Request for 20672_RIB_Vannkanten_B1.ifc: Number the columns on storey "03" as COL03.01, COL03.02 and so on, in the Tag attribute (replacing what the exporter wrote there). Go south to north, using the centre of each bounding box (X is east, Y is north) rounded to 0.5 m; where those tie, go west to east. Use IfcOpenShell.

First a look at what the model holds.

```python
import ifcopenshell
import ifcopenshell.util.element
import ifcopenshell.util.placement

model = ifcopenshell.open("20672_RIB_Vannkanten_B1.ifc")
print(model.schema)
storey = next(s for s in model.by_type("IfcBuildingStorey") if s.Name == "03")
columns = [e for e in ifcopenshell.util.element.get_decomposition(storey) if e.is_a("IfcColumn")]
for e in sorted(columns, key=lambda e: e.id()):
    origin = ifcopenshell.util.placement.get_local_placement(e.ObjectPlacement)[:3, 3]
    print(e.id(), e.Tag, e.Name, origin.round(2) + 0.0, sep=" | ")
```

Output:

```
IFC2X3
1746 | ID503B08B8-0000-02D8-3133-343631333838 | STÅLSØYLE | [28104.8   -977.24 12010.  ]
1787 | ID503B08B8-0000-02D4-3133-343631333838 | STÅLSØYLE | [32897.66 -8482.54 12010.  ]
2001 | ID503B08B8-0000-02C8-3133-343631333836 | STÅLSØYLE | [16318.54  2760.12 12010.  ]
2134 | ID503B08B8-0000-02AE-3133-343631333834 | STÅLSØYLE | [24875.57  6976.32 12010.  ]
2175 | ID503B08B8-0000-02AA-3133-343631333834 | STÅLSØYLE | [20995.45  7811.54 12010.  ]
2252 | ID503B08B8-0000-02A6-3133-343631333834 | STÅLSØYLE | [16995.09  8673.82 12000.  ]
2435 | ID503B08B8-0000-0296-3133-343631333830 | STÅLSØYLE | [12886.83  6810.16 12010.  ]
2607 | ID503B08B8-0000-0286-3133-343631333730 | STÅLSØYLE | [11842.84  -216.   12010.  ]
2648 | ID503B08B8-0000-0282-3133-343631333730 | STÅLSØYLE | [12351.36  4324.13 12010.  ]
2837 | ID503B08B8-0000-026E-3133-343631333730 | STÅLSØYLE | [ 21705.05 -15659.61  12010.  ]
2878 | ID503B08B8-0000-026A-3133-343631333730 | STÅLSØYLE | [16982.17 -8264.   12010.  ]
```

```python
import ifcopenshell
import ifcopenshell.geom
import ifcopenshell.util.element
import ifcopenshell.util.shape

model = ifcopenshell.open("20672_RIB_Vannkanten_B1.ifc")
settings = ifcopenshell.geom.settings()
settings.set("use-world-coords", True)


def centre(element):
    shape = ifcopenshell.geom.create_shape(settings, element)
    return ifcopenshell.util.shape.get_bbox_centroid(shape.geometry)


storey = next(s for s in model.by_type("IfcBuildingStorey") if s.Name == "03")
columns = [e for e in ifcopenshell.util.element.get_decomposition(storey) if e.is_a("IfcColumn")]

# Insertion points can sit at a corner or the storey origin, so sort by the geometry (in metres).
centres = {e: centre(e) for e in columns}
columns.sort(key=lambda e: (round(centres[e][1] / 0.5), centres[e][0]))

for i, e in enumerate(columns, start=1):
    number = f"COL03.{i:02d}"
    e.Tag = number
    print(e.id(), number)

model.write("20672_RIB_Vannkanten_B1_v2.ifc")
```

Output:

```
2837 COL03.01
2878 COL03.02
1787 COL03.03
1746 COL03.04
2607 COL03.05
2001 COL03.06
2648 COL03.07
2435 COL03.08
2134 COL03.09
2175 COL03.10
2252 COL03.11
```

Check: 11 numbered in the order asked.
